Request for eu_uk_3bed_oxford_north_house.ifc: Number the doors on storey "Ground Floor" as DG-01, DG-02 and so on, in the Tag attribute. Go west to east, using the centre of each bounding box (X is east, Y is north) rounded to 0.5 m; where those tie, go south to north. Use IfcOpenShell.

First a look at what the model holds.

```python
import ifcopenshell
import ifcopenshell.util.element
import ifcopenshell.util.placement

model = ifcopenshell.open("eu_uk_3bed_oxford_north_house.ifc")
print(model.schema)
storey = next(s for s in model.by_type("IfcBuildingStorey") if s.Name == "Ground Floor")
doors = [e for e in ifcopenshell.util.element.get_decomposition(storey) if e.is_a("IfcDoor")]
for e in sorted(doors, key=lambda e: e.id()):
    origin = ifcopenshell.util.placement.get_local_placement(e.ObjectPlacement)[:3, 3]
    print(e.id(), e.Tag, e.Name, origin.round(2) + 0.0, sep=" | ")
```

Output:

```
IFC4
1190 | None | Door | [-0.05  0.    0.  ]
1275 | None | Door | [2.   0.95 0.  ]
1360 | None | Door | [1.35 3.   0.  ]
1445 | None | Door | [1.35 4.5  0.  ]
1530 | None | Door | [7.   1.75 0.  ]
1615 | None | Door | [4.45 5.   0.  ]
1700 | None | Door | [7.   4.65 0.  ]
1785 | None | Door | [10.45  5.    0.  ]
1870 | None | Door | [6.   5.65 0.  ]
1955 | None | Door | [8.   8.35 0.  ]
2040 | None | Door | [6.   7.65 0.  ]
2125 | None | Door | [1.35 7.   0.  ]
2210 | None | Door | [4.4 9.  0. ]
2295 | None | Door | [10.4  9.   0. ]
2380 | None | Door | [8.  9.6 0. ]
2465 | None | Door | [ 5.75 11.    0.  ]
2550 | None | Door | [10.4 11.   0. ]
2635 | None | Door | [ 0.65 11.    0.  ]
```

```python
import ifcopenshell
import ifcopenshell.geom
import ifcopenshell.util.element
import ifcopenshell.util.shape

model = ifcopenshell.open("eu_uk_3bed_oxford_north_house.ifc")
settings = ifcopenshell.geom.settings()
settings.set("use-world-coords", True)


def centre(element):
    shape = ifcopenshell.geom.create_shape(settings, element)
    return ifcopenshell.util.shape.get_bbox_centroid(shape.geometry)


storey = next(s for s in model.by_type("IfcBuildingStorey") if s.Name == "Ground Floor")
doors = [e for e in ifcopenshell.util.element.get_decomposition(storey) if e.is_a("IfcDoor")]

# Insertion points can sit at a corner or the storey origin, so sort by the geometry (in metres).
centres = {e: centre(e) for e in doors}
doors.sort(key=lambda e: (round(centres[e][0] / 0.5), centres[e][1]))

for i, e in enumerate(doors, start=1):
    number = f"DG-{i:02d}"
    e.Tag = number
    print(e.id(), number)

model.write("eu_uk_3bed_oxford_north_house_edited.ifc")
```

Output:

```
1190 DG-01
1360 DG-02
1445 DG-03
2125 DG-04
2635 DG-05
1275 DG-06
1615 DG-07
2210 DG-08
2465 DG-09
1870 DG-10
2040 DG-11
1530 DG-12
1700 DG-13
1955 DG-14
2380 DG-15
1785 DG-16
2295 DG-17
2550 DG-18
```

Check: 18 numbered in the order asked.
